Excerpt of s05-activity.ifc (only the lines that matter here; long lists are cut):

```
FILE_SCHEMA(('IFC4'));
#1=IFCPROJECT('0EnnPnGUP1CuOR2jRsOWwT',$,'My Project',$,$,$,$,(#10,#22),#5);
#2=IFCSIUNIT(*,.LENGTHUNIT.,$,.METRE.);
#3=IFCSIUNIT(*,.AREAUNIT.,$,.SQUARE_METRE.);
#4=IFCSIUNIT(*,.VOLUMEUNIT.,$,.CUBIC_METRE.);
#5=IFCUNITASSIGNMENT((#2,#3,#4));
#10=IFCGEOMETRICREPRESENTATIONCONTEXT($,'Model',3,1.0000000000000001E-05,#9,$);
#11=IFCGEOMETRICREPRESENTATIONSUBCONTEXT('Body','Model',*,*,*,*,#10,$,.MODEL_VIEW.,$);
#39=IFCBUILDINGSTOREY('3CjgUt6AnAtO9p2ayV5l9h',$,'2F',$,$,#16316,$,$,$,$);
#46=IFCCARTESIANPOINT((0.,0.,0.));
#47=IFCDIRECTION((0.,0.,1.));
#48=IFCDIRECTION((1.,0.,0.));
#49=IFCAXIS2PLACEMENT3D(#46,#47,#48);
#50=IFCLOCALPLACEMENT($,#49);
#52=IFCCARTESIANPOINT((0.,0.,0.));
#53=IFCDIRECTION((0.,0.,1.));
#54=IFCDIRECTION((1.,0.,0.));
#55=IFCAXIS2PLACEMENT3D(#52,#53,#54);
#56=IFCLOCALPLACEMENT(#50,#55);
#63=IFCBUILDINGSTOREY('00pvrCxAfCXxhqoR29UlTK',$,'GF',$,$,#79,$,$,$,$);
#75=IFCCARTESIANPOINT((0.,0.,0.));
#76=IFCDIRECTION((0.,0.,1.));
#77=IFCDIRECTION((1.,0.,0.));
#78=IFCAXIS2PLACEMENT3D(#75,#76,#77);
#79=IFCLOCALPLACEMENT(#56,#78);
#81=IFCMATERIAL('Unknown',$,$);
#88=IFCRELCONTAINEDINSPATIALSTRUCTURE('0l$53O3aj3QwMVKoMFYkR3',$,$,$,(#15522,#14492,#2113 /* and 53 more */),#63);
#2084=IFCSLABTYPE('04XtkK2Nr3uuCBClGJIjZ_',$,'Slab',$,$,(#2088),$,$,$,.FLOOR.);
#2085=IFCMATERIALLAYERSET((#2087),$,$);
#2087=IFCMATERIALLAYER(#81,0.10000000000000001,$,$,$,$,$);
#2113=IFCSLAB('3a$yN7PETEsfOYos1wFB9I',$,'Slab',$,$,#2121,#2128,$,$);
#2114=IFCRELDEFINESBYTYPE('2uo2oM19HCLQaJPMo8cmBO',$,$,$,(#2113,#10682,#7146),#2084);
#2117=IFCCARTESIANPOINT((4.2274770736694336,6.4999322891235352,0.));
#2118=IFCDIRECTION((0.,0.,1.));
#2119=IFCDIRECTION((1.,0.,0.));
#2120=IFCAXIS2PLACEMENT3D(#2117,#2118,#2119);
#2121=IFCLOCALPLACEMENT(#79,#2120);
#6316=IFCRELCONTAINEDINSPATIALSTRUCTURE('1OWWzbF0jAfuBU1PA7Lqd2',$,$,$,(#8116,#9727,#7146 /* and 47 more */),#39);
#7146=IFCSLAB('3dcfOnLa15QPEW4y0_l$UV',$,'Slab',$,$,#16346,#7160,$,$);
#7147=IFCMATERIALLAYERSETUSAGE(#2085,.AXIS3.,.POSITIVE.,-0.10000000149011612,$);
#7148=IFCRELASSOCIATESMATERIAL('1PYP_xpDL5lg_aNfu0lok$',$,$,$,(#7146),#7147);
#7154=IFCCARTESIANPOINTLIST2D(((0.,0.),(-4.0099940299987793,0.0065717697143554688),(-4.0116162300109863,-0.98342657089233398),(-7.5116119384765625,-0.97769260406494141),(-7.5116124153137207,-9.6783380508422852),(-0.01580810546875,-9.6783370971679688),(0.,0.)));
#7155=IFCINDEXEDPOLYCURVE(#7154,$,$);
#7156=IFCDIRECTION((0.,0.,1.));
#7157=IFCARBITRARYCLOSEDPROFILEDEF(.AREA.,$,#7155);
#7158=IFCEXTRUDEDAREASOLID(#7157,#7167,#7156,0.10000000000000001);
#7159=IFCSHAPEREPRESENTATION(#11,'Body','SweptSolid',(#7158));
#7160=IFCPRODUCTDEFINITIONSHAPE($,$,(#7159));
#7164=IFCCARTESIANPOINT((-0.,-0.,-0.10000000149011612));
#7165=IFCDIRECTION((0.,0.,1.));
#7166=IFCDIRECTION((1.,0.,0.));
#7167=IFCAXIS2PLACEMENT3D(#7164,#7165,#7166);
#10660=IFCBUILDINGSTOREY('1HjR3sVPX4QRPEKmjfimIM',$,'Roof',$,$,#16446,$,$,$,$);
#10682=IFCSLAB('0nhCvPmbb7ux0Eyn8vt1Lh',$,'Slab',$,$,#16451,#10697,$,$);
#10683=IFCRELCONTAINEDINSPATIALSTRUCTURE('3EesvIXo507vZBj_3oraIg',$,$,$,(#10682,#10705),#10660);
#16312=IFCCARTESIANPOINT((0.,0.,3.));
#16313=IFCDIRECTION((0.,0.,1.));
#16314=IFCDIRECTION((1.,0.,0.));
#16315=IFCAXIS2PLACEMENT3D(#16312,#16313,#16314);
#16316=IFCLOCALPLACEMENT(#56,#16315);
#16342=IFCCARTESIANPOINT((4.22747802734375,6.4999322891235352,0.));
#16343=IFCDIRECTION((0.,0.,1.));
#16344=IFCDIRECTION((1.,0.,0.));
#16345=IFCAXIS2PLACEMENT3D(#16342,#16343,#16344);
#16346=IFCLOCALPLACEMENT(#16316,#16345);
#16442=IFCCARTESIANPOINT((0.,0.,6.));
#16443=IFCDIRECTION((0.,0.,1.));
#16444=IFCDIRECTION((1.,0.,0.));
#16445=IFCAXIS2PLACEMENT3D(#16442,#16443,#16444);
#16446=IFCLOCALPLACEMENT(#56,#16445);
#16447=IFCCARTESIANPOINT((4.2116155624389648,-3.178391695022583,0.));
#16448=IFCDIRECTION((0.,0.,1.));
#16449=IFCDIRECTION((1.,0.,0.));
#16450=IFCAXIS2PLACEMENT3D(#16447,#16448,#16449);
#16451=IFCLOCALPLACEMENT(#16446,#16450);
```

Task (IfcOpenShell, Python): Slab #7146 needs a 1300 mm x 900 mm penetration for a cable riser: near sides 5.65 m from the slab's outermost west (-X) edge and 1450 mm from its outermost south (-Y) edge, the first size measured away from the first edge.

```python
import numpy as np
import ifcopenshell
import ifcopenshell.api.feature
import ifcopenshell.api.geometry
import ifcopenshell.api.root
import ifcopenshell.geom
import ifcopenshell.util.placement
import ifcopenshell.util.representation
import ifcopenshell.util.shape
import ifcopenshell.util.unit

model = ifcopenshell.open("s05-activity.ifc")
unit_scale = ifcopenshell.util.unit.calculate_unit_scale(model)
settings = ifcopenshell.geom.settings()


def volume(element):
    """Net volume in cubic metres, openings subtracted."""
    shape = ifcopenshell.geom.create_shape(settings, element)
    return ifcopenshell.util.shape.get_volume(shape.geometry)


slab = model.by_id(7146)
before = volume(slab)

# Extent in the slab's own axes, in metres. The edges named are its -X and -Y sides.
slab_shape = ifcopenshell.geom.create_shape(settings, slab)
vertices = ifcopenshell.util.shape.get_vertices(slab_shape.geometry)
x_min, y_min, bottom = vertices.min(axis=0)
top = vertices[:, 2].max()

opening = ifcopenshell.api.root.create_entity(model, ifc_class="IfcOpeningElement", name="Cable riser opening", predefined_type="OPENING")
context = ifcopenshell.util.representation.get_context(model, "Model", "Body", "MODEL_VIEW")
width, depth = 1.3, 0.9
outline = [(0.0, 0.0), (width, 0.0), (width, depth), (0.0, depth), (0.0, 0.0)]
# Overshoot both faces by 50 mm so the cut is clean.
shape = ifcopenshell.api.geometry.add_slab_representation(
    model, context=context, depth=top - bottom + 0.1, polyline=outline
)
ifcopenshell.api.geometry.assign_representation(model, product=opening, representation=shape)

matrix = ifcopenshell.util.placement.get_local_placement(slab.ObjectPlacement)
matrix[:, 3] = matrix @ np.append(np.array([x_min + 5.65, y_min + 1.45, bottom - 0.05]) / unit_scale, 1.0)
ifcopenshell.api.geometry.edit_object_placement(model, product=opening, matrix=matrix, is_si=False)
ifcopenshell.api.feature.add_feature(model, feature=opening, element=slab)

after = volume(slab)

print(f"slab volume {before:.3f} -> {after:.3f} m3")

model.write("s05-activity_v2.ifc")
```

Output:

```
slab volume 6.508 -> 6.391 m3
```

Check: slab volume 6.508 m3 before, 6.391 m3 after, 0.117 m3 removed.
